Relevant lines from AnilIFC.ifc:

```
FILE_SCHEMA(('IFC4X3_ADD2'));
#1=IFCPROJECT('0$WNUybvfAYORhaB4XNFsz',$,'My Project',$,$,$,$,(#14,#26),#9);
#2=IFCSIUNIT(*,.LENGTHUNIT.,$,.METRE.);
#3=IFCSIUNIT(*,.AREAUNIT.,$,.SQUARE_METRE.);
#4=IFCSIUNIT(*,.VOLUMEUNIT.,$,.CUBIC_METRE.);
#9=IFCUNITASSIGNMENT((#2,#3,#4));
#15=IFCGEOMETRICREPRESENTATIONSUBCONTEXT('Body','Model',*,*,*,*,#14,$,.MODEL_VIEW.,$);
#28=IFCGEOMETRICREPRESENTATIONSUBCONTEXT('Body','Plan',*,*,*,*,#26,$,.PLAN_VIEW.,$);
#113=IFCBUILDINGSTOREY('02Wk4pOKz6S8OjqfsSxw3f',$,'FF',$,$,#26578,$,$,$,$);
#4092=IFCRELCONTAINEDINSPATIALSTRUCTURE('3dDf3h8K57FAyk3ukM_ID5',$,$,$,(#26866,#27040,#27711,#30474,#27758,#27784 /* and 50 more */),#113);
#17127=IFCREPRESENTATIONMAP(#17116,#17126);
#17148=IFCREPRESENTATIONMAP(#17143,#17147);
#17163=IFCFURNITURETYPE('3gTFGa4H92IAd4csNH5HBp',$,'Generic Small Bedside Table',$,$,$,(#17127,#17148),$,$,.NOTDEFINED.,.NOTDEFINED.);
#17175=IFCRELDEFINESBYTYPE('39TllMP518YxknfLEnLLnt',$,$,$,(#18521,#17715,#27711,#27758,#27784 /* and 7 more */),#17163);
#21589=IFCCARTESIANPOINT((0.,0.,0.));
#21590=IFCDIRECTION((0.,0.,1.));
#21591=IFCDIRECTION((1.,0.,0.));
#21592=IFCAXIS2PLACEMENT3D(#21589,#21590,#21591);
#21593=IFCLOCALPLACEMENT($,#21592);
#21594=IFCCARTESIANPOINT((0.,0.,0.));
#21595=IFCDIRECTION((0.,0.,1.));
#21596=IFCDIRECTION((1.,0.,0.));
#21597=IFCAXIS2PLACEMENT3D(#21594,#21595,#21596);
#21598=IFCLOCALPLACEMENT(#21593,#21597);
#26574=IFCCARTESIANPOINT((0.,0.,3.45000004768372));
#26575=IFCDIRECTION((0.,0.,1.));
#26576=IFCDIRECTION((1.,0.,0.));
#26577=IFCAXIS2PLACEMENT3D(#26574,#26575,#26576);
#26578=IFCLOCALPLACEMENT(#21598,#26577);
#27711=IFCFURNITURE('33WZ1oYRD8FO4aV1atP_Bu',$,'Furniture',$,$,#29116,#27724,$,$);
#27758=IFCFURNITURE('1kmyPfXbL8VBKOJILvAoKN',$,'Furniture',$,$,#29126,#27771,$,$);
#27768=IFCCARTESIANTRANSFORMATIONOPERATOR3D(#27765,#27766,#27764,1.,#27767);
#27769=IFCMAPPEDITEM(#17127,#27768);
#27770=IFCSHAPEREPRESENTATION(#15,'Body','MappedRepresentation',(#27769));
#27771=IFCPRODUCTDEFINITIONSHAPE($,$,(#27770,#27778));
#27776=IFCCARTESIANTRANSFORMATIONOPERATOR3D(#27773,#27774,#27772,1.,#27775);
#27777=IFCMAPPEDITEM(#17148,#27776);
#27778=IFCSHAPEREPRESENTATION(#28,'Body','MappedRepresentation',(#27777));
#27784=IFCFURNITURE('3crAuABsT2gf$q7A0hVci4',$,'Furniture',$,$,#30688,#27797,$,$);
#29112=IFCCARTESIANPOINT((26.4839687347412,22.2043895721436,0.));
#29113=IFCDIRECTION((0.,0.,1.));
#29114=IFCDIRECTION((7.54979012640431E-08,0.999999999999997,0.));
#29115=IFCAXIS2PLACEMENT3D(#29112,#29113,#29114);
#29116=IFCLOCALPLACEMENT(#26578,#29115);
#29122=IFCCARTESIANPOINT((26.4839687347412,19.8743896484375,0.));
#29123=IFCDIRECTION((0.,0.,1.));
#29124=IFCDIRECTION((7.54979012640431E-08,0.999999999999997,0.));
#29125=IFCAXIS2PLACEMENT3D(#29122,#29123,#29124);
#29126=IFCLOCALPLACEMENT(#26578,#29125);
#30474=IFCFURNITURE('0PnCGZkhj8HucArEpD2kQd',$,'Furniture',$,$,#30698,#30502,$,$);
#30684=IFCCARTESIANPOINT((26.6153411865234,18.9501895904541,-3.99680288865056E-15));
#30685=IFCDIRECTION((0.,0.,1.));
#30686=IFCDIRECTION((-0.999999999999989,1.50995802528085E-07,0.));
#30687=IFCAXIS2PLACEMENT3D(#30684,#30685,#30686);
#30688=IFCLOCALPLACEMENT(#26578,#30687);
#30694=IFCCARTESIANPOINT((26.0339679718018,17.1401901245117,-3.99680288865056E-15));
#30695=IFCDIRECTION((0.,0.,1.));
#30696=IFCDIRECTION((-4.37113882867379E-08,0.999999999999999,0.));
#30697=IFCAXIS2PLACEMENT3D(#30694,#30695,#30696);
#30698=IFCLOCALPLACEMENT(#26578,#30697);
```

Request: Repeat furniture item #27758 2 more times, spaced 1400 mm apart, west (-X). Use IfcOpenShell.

```python
import numpy as np
import ifcopenshell
import ifcopenshell.api.geometry
import ifcopenshell.api.root
import ifcopenshell.util.element
import ifcopenshell.util.placement
import ifcopenshell.util.unit

model = ifcopenshell.open("AnilIFC.ifc")
unit_scale = ifcopenshell.util.unit.calculate_unit_scale(model)

source = model.by_guid("1kmyPfXbL8VBKOJILvAoKN")
base = ifcopenshell.util.placement.get_local_placement(source.ObjectPlacement)
step = np.array([-1.0, 0.0, 0.0]) * 1.4 / unit_scale

for i in range(1, 3):
    copy = ifcopenshell.api.root.copy_class(model, product=source)
    copy.Representation = ifcopenshell.util.element.copy_deep(
        model, source.Representation, exclude=["IfcGeometricRepresentationContext", "IfcRepresentationMap"]
    )
    matrix = base.copy()
    matrix[:3, 3] += i * step
    print("added at", matrix[:3, 3].round(3) + 0.0)
    ifcopenshell.api.geometry.edit_object_placement(model, product=copy, matrix=matrix, is_si=False)

model.write("AnilIFC_rev.ifc")
```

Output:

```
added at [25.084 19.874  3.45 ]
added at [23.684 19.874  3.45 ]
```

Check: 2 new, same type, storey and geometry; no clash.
